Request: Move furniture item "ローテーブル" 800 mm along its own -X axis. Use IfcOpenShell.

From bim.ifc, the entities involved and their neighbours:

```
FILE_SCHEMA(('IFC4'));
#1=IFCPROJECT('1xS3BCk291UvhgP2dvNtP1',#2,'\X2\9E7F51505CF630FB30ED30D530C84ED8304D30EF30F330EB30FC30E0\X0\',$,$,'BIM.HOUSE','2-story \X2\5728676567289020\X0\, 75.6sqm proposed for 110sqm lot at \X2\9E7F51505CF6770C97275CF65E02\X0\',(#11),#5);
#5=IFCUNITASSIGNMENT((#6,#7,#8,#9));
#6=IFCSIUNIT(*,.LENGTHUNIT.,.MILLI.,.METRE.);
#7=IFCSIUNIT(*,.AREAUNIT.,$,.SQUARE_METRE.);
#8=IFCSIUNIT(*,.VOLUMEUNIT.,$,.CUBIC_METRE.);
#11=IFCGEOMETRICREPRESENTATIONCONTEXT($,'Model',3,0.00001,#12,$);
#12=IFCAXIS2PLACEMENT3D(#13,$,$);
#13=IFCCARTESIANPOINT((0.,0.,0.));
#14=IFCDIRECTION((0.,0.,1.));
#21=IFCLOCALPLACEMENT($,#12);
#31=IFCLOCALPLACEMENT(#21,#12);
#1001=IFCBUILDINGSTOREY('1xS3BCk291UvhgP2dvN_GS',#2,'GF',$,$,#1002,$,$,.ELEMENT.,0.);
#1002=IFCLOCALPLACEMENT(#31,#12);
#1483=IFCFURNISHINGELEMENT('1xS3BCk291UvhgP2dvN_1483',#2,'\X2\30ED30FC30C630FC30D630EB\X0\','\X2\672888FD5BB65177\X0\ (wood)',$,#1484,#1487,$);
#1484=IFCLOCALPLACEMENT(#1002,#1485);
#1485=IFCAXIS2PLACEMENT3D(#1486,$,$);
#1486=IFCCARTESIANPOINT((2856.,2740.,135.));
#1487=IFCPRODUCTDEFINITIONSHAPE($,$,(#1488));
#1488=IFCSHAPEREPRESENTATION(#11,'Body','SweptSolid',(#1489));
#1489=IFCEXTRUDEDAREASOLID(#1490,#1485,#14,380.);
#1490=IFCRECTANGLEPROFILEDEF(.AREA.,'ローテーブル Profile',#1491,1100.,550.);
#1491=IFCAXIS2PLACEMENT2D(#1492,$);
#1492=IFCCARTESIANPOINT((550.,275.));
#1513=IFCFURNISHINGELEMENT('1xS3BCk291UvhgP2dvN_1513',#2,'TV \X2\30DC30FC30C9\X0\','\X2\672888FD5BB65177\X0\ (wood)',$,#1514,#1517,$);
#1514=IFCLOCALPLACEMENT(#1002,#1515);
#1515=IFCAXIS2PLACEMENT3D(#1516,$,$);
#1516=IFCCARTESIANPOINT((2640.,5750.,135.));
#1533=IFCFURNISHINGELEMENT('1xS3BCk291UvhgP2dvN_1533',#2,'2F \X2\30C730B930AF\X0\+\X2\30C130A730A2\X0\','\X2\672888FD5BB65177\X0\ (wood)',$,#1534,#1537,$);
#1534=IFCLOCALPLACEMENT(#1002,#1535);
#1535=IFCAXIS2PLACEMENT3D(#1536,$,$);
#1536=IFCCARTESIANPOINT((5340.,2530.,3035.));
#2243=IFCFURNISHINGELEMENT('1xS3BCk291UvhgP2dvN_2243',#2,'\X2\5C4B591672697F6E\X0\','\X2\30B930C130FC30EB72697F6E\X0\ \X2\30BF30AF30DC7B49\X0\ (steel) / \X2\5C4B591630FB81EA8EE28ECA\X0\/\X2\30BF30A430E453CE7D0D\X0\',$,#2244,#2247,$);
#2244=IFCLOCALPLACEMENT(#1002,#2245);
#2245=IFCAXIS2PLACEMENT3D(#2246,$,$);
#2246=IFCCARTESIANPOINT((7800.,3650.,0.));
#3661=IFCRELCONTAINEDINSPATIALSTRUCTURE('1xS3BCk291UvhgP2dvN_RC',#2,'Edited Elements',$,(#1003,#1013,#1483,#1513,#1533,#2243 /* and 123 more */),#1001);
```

```python
import ifcopenshell
import ifcopenshell.api.geometry
import ifcopenshell.util.placement

model = ifcopenshell.open("bim.ifc")

item = model.by_id(1483)
matrix = ifcopenshell.util.placement.get_local_placement(item.ObjectPlacement)
matrix[:3, 3] -= matrix[:3, 0] * 800.0
ifcopenshell.api.geometry.edit_object_placement(model, product=item, matrix=matrix, is_si=False)

print(ifcopenshell.util.placement.get_local_placement(item.ObjectPlacement).round(3) + 0.0)

model.write("bim_v2.ifc")
```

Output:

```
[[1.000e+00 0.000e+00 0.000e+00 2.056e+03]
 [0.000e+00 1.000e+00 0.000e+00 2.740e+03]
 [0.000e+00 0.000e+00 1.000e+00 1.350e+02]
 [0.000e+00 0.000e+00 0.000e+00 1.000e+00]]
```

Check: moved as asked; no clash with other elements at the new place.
